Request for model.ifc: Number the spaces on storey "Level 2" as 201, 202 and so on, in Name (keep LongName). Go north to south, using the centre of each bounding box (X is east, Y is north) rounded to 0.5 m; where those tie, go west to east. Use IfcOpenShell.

First a look at what the model holds.

```python
import ifcopenshell
import ifcopenshell.util.element
import ifcopenshell.util.placement

model = ifcopenshell.open("model.ifc")
print(model.schema)
storey = next(s for s in model.by_type("IfcBuildingStorey") if s.Name == "Level 2")
spaces = [e for e in ifcopenshell.util.element.get_decomposition(storey) if e.is_a("IfcSpace")]
for e in sorted(spaces, key=lambda e: e.id()):
    origin = ifcopenshell.util.placement.get_local_placement(e.ObjectPlacement)[:3, 3]
    print(e.id(), e.Name, e.LongName, origin.round(2) + 0.0, sep=" | ")
```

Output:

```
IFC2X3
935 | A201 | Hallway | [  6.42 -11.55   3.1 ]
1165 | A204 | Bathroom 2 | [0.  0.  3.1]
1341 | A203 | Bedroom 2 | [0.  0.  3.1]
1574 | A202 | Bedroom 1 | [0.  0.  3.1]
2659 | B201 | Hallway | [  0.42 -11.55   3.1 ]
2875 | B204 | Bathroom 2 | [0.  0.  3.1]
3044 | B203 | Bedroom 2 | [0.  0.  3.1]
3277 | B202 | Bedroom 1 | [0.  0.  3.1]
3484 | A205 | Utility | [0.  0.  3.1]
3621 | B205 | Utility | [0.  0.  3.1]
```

```python
import ifcopenshell
import ifcopenshell.geom
import ifcopenshell.util.element
import ifcopenshell.util.shape

model = ifcopenshell.open("model.ifc")
settings = ifcopenshell.geom.settings()
settings.set("use-world-coords", True)


def centre(element):
    shape = ifcopenshell.geom.create_shape(settings, element)
    return ifcopenshell.util.shape.get_bbox_centroid(shape.geometry)


storey = next(s for s in model.by_type("IfcBuildingStorey") if s.Name == "Level 2")
spaces = [e for e in ifcopenshell.util.element.get_decomposition(storey) if e.is_a("IfcSpace")]

# Insertion points can sit at a corner or the storey origin, so sort by the geometry (in metres).
centres = {e: centre(e) for e in spaces}
spaces.sort(key=lambda e: (-round(centres[e][1] / 0.5), centres[e][0]))

for i, e in enumerate(spaces, start=1):
    number = f"2{i:02d}"
    e.Name = number
    print(e.id(), number)

model.write("model_updated.ifc")
```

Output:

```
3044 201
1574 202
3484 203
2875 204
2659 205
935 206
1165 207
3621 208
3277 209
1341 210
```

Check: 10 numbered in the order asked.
